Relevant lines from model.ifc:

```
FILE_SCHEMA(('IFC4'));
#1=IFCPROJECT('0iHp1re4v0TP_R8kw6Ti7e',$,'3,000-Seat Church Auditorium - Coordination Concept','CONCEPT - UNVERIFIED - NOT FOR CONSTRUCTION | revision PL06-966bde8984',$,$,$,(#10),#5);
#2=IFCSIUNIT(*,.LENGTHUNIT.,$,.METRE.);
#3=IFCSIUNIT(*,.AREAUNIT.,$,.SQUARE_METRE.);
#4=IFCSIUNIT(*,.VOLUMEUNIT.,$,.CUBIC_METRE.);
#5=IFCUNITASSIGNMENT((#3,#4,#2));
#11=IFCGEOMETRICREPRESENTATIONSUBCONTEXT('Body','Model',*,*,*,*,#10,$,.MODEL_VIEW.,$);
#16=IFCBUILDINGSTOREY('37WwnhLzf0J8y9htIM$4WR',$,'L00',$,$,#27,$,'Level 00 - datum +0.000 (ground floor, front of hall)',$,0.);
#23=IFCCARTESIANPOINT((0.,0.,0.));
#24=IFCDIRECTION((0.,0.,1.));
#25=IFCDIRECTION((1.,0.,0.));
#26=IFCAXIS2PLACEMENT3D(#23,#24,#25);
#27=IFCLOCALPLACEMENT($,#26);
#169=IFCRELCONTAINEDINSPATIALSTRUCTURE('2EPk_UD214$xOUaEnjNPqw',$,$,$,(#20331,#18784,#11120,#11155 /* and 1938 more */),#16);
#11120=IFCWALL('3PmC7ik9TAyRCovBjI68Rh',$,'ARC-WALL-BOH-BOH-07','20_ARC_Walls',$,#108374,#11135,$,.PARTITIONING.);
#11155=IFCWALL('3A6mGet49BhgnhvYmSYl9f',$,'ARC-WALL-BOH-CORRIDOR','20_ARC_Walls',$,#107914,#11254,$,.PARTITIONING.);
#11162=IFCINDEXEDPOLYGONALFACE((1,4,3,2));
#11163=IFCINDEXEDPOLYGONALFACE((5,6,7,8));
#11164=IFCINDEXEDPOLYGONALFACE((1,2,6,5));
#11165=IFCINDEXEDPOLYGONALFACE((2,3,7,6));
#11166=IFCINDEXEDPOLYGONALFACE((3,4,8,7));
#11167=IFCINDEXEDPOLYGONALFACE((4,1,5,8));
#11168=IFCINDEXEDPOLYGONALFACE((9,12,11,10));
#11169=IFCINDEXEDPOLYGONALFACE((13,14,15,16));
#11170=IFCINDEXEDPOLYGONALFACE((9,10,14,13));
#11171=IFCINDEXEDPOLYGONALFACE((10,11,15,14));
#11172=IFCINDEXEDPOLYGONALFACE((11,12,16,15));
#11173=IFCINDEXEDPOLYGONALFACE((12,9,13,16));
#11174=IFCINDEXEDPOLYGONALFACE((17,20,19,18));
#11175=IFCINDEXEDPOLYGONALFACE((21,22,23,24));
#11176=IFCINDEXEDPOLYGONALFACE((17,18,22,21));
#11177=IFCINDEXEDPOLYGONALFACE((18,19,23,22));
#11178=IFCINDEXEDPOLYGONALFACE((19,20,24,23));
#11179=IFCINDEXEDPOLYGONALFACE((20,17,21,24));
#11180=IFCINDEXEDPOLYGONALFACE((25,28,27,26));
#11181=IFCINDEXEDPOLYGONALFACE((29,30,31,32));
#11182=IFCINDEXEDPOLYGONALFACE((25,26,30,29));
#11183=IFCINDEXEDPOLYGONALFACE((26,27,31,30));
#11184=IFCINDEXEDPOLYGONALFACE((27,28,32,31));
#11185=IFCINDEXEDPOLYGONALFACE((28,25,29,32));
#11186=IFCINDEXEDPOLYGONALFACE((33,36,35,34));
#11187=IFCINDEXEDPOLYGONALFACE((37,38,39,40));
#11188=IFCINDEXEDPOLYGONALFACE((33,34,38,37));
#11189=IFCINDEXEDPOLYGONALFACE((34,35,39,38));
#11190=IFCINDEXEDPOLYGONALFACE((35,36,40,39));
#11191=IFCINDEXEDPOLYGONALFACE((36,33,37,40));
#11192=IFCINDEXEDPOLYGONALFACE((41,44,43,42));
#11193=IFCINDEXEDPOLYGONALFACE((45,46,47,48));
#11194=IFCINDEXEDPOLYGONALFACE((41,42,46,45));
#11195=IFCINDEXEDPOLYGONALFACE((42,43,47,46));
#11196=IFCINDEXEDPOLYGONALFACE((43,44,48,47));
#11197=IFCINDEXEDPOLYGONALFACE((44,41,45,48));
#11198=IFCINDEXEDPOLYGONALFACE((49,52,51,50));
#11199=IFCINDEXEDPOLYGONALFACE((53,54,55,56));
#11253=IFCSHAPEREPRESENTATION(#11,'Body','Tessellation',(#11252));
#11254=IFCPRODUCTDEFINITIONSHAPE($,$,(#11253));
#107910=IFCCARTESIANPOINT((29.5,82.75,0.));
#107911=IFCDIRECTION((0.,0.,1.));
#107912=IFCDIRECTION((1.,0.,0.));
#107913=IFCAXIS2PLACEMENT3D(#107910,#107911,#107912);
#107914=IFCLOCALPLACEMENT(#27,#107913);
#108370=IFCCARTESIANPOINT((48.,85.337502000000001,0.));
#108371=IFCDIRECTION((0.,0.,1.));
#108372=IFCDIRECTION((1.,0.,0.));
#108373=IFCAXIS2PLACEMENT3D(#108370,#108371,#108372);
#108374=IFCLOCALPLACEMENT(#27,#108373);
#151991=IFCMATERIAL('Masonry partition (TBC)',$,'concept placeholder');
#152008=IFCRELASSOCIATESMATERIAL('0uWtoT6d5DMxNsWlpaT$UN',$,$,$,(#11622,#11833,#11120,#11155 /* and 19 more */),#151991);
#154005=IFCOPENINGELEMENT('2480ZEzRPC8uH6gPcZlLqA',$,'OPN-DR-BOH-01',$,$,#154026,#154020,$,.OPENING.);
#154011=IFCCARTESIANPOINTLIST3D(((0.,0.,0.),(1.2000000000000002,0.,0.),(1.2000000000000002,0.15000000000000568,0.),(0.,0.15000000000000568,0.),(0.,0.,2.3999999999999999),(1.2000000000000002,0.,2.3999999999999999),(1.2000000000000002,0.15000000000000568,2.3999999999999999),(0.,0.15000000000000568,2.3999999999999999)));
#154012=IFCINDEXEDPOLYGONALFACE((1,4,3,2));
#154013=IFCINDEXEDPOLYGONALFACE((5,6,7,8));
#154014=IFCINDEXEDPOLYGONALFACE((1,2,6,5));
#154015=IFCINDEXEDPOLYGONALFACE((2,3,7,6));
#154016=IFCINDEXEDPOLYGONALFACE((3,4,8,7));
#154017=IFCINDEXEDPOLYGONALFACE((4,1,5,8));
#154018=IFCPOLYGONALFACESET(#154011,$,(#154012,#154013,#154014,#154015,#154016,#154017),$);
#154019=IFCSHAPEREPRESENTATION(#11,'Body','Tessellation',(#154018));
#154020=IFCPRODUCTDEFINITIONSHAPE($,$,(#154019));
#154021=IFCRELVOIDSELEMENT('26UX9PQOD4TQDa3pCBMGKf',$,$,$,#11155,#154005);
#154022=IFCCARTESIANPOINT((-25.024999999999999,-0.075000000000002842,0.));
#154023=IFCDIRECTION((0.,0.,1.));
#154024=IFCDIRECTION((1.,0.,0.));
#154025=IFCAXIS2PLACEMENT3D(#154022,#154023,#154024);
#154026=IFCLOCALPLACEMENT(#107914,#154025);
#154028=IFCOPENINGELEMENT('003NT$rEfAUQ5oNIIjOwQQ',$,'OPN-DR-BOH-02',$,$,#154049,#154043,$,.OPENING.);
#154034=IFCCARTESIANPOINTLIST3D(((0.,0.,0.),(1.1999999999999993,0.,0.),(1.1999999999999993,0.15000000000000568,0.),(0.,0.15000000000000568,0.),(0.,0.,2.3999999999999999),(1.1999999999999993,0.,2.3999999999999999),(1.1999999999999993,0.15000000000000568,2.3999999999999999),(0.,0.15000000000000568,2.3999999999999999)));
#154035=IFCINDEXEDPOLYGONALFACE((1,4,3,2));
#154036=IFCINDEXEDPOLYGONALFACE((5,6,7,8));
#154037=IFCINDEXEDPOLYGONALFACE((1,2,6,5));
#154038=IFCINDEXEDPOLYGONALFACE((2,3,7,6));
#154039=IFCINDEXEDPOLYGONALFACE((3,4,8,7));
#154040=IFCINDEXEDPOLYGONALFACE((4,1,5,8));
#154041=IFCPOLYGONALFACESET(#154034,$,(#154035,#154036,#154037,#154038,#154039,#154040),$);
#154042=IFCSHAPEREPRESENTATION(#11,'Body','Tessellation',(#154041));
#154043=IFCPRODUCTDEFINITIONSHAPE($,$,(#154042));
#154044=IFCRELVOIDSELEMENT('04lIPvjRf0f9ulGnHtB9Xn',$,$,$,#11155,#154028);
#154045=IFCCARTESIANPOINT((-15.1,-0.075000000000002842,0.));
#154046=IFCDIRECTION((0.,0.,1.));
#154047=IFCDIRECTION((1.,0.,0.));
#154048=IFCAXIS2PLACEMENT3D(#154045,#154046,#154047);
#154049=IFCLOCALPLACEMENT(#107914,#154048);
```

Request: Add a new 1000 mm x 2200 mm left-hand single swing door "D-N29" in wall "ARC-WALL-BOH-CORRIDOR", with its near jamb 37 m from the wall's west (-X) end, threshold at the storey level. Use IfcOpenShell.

```python
import numpy as np
import ifcopenshell
import ifcopenshell.api.feature
import ifcopenshell.api.geometry
import ifcopenshell.api.root
import ifcopenshell.api.spatial
import ifcopenshell.geom
import ifcopenshell.util.element
import ifcopenshell.util.placement
import ifcopenshell.util.representation
import ifcopenshell.util.shape
import ifcopenshell.util.unit

model = ifcopenshell.open("model.ifc")
unit_scale = ifcopenshell.util.unit.calculate_unit_scale(model)
settings = ifcopenshell.geom.settings()


def volume(element):
    """Net volume in cubic metres, openings subtracted."""
    shape = ifcopenshell.geom.create_shape(settings, element)
    return ifcopenshell.util.shape.get_volume(shape.geometry)


wall = model.by_guid("3A6mGet49BhgnhvYmSYl9f")
storey = ifcopenshell.util.element.get_container(wall, ifc_class="IfcBuildingStorey")
context = ifcopenshell.util.representation.get_context(model, "Model", "Body", "MODEL_VIEW")
before = volume(wall)

width, height, from_end, sill = 1, 2.2, 37, 0.0  # metres

# The wall runs along its own X axis, and the end named is its -X end.
wall_shape = ifcopenshell.geom.create_shape(settings, wall)
x, y, z = ifcopenshell.util.shape.get_vertices(wall_shape.geometry).T
start = x.min() + from_end
face, thickness = float(y.min()), float(y.max() - y.min())
wall_matrix = ifcopenshell.util.placement.get_local_placement(wall.ObjectPlacement)
level = ifcopenshell.util.placement.get_local_placement(storey.ObjectPlacement)[2, 3]


def in_wall(x, y):
    """Placement at x, y metres in the wall's axes, at sill height."""
    matrix = wall_matrix.copy()
    matrix[:, 3] = wall_matrix @ np.array([x / unit_scale, y / unit_scale, 0.0, 1.0])
    matrix[2, 3] = level + sill / unit_scale
    return matrix


# Opening: a box that overshoots both wall faces by 50 mm.
opening = ifcopenshell.api.root.create_entity(model, ifc_class="IfcOpeningElement", predefined_type="OPENING")
box = ifcopenshell.api.geometry.add_wall_representation(
    model, context=context, length=width, height=height, thickness=thickness + 0.1
)
ifcopenshell.api.geometry.assign_representation(model, product=opening, representation=box)
ifcopenshell.api.geometry.edit_object_placement(model, product=opening, matrix=in_wall(start, face - 0.05), is_si=False)
ifcopenshell.api.feature.add_feature(model, feature=opening, element=wall)

door = ifcopenshell.api.root.create_entity(model, ifc_class="IfcDoor", name="D-N29", predefined_type="DOOR")
door.OverallWidth, door.OverallHeight = width / unit_scale, height / unit_scale
door.OperationType = "SINGLE_SWING_LEFT"
body = ifcopenshell.api.geometry.add_door_representation(
    model,
    context=context,
    overall_width=door.OverallWidth,
    overall_height=door.OverallHeight,
    operation_type="SINGLE_SWING_LEFT",
    lining_properties={"LiningDepth": thickness / unit_scale, "ThresholdDepth": thickness / unit_scale},
)
ifcopenshell.api.geometry.assign_representation(model, product=door, representation=body)
ifcopenshell.api.spatial.assign_container(model, products=[door], relating_structure=storey)
ifcopenshell.api.feature.add_filling(model, opening=opening, element=door)

# The lining spans the wall, so the door starts at the wall face.
ifcopenshell.api.geometry.edit_object_placement(model, product=door, matrix=in_wall(start, face), is_si=False)

after = volume(wall)

print(f"wall volume {before:.3f} -> {after:.3f} m3")

model.write("model-out.ifc")
```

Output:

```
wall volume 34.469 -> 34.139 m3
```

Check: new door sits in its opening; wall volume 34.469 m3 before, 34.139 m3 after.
